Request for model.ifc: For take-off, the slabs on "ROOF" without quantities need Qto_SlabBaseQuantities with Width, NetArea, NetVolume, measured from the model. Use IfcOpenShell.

First a look at what the model holds.

```python
import ifcopenshell
import ifcopenshell.util.element
import ifcopenshell.util.unit

model = ifcopenshell.open("model.ifc")
print(model.schema)
for unit_type in ("LENGTHUNIT", "AREAUNIT", "VOLUMEUNIT"):
    print(unit_type, ifcopenshell.util.unit.calculate_unit_scale(model, unit_type))
storey = next(s for s in model.by_type("IfcBuildingStorey") if s.Name == "ROOF")
slabs = [e for e in ifcopenshell.util.element.get_decomposition(storey) if e.is_a("IfcSlab")]
for e in sorted(slabs, key=lambda e: e.id()):
    print(e.id(), e.is_a(), e.Name, list(ifcopenshell.util.element.get_psets(e, qtos_only=True)), sep=" | ")
```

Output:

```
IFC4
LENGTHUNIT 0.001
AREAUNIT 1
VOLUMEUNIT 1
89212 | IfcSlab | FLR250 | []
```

```python
import ifcopenshell
import ifcopenshell.api.pset
import ifcopenshell.geom
import ifcopenshell.util.element
import ifcopenshell.util.shape
import ifcopenshell.util.unit

model = ifcopenshell.open("model.ifc")
unit_scale = ifcopenshell.util.unit.calculate_unit_scale(model)
area_scale = ifcopenshell.util.unit.calculate_unit_scale(model, "AREAUNIT")
volume_scale = ifcopenshell.util.unit.calculate_unit_scale(model, "VOLUMEUNIT")
settings = ifcopenshell.geom.settings()

storey = next(s for s in model.by_type("IfcBuildingStorey") if s.Name == "ROOF")
slabs = [e for e in ifcopenshell.util.element.get_decomposition(storey) if e.is_a("IfcSlab")]

for e in sorted(slabs, key=lambda e: e.id()):
    if ifcopenshell.util.element.get_psets(e, qtos_only=True, should_inherit=False):
        continue
    # Geometry comes back in metres, in the element's own axes.
    shape = ifcopenshell.geom.create_shape(settings, e)
    values = {
        "Width": ifcopenshell.util.shape.get_z(shape.geometry) / unit_scale,
        "NetArea": ifcopenshell.util.shape.get_footprint_area(shape.geometry) / area_scale,
        "NetVolume": ifcopenshell.util.shape.get_volume(shape.geometry) / volume_scale,
    }
    qto = ifcopenshell.api.pset.add_qto(model, product=e, name="Qto_SlabBaseQuantities")
    ifcopenshell.api.pset.edit_qto(model, qto=qto, properties=values)
    print(e.id(), {k: round(v, 3) for k, v in values.items()})

model.write("model_rev.ifc")
```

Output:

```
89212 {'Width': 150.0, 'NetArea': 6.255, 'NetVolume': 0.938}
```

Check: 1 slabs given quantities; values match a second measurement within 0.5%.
